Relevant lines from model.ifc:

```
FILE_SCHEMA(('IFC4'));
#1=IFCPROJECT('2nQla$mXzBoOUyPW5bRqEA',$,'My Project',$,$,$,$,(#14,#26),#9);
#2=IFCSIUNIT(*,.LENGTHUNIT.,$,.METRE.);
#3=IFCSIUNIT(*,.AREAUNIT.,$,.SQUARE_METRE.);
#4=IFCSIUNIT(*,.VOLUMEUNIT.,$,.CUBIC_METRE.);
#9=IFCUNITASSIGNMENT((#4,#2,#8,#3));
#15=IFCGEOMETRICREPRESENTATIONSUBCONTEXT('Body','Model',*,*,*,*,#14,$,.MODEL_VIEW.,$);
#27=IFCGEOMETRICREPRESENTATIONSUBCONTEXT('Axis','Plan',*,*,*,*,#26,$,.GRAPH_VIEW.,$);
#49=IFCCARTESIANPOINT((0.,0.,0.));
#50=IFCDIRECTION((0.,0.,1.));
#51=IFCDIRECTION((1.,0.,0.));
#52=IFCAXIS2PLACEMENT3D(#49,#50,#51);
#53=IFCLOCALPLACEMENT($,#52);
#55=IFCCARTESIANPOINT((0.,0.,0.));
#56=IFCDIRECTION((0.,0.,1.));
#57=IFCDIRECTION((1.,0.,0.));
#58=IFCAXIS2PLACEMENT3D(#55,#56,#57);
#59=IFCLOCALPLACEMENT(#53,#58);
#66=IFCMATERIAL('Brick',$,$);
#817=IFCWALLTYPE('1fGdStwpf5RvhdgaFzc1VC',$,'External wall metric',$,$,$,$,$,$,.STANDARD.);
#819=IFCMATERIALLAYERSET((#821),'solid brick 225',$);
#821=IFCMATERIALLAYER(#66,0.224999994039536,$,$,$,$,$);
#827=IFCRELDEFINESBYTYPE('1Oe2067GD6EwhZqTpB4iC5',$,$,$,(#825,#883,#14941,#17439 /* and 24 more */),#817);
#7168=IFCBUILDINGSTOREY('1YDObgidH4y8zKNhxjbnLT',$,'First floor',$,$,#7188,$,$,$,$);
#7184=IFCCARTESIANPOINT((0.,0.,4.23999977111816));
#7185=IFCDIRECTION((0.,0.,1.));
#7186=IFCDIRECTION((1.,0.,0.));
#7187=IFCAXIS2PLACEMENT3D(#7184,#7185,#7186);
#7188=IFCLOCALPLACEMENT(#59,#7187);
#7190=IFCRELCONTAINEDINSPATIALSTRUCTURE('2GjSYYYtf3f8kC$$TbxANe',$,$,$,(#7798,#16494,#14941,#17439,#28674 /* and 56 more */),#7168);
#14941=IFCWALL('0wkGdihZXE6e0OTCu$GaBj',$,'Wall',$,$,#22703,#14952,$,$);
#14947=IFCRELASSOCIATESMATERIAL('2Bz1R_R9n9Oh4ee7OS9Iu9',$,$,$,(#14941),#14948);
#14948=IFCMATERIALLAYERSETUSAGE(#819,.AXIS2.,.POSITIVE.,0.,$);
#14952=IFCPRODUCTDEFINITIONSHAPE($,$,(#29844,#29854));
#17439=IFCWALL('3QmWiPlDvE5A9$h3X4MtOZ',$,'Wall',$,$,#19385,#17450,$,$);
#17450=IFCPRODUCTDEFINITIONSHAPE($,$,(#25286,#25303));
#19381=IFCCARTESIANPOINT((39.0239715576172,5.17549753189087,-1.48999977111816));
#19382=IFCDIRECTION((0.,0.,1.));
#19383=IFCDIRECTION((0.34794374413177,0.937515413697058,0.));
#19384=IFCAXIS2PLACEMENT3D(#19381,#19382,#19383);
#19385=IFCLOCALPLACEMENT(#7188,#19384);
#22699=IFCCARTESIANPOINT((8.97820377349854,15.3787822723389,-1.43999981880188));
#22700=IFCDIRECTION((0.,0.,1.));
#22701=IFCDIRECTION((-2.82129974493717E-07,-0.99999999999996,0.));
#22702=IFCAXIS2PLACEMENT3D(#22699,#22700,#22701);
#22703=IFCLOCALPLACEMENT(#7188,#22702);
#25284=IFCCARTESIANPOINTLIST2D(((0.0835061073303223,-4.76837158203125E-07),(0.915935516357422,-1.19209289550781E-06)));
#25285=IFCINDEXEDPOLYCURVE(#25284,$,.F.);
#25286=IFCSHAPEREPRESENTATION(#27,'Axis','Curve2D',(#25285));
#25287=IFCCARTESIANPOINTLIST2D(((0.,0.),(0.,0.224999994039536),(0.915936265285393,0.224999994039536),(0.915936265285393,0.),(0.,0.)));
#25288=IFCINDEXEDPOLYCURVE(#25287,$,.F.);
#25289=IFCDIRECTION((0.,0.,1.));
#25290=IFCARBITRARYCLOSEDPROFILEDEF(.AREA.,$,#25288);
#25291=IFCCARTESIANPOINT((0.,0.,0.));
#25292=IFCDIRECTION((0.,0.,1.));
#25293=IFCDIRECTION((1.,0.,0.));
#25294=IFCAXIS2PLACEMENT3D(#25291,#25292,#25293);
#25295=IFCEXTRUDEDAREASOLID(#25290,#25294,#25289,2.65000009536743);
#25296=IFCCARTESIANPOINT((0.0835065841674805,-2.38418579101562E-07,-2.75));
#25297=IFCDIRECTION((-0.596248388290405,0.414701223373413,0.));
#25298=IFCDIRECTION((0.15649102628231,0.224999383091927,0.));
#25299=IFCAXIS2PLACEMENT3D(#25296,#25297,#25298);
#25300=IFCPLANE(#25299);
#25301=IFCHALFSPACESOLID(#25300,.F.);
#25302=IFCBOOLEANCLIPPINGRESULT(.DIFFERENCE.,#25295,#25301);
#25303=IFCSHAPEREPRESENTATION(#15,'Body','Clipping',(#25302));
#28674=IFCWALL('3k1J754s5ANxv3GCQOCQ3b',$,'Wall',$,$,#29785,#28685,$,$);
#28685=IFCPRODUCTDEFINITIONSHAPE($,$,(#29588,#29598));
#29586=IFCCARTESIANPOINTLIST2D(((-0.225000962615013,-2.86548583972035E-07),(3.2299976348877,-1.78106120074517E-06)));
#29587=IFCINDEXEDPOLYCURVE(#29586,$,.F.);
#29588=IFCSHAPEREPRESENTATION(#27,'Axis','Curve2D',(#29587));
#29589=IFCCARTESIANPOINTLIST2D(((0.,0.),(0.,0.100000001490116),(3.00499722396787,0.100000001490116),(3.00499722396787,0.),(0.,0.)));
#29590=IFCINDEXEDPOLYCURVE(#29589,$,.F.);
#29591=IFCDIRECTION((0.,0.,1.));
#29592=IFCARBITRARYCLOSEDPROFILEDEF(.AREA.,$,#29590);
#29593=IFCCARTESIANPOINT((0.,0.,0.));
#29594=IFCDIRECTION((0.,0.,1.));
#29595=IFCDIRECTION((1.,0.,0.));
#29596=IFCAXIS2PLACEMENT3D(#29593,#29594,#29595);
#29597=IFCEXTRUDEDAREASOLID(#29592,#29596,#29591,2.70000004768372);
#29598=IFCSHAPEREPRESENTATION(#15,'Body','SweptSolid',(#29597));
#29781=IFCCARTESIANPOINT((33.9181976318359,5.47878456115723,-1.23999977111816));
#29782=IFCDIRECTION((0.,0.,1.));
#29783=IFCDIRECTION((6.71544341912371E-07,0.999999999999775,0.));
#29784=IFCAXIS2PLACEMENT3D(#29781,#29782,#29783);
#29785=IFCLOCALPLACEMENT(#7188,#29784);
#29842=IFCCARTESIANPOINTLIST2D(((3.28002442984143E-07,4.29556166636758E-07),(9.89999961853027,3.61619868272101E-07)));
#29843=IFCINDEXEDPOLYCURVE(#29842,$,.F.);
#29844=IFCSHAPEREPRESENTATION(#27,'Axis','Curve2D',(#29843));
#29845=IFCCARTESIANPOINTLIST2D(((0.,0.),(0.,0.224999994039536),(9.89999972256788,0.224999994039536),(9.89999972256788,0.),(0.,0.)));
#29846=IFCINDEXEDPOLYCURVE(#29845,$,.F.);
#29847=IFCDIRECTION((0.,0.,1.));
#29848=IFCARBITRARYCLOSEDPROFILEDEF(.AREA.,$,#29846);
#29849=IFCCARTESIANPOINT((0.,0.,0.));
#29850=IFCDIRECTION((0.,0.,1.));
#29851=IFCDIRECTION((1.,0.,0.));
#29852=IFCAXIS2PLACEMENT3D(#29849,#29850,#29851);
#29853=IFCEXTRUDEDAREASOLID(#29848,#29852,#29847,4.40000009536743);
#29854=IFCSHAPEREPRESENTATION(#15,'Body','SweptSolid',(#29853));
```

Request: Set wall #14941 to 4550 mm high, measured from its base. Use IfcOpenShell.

```python
import ifcopenshell
import ifcopenshell.geom
import ifcopenshell.util.representation
import ifcopenshell.util.shape
import ifcopenshell.util.unit

model = ifcopenshell.open("model.ifc")
unit_scale = ifcopenshell.util.unit.calculate_unit_scale(model)
settings = ifcopenshell.geom.settings()


def volume(element):
    """Net volume in cubic metres, openings subtracted."""
    shape = ifcopenshell.geom.create_shape(settings, element)
    return ifcopenshell.util.shape.get_volume(shape.geometry)


wall = model.by_id(14941)
before = volume(wall)

body = ifcopenshell.util.representation.get_representation(wall, "Model", "Body")
solid = body.Items[0]
old_height = solid.Depth
solid.Depth = 4.55 / unit_scale
after = volume(wall)

print(f"height {old_height:g} -> {solid.Depth:g}, volume {before:.3f} -> {after:.3f} m3")

model.write("model_rev.ifc")
```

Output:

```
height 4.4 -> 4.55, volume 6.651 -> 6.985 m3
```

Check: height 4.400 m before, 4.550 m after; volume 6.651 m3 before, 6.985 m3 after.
